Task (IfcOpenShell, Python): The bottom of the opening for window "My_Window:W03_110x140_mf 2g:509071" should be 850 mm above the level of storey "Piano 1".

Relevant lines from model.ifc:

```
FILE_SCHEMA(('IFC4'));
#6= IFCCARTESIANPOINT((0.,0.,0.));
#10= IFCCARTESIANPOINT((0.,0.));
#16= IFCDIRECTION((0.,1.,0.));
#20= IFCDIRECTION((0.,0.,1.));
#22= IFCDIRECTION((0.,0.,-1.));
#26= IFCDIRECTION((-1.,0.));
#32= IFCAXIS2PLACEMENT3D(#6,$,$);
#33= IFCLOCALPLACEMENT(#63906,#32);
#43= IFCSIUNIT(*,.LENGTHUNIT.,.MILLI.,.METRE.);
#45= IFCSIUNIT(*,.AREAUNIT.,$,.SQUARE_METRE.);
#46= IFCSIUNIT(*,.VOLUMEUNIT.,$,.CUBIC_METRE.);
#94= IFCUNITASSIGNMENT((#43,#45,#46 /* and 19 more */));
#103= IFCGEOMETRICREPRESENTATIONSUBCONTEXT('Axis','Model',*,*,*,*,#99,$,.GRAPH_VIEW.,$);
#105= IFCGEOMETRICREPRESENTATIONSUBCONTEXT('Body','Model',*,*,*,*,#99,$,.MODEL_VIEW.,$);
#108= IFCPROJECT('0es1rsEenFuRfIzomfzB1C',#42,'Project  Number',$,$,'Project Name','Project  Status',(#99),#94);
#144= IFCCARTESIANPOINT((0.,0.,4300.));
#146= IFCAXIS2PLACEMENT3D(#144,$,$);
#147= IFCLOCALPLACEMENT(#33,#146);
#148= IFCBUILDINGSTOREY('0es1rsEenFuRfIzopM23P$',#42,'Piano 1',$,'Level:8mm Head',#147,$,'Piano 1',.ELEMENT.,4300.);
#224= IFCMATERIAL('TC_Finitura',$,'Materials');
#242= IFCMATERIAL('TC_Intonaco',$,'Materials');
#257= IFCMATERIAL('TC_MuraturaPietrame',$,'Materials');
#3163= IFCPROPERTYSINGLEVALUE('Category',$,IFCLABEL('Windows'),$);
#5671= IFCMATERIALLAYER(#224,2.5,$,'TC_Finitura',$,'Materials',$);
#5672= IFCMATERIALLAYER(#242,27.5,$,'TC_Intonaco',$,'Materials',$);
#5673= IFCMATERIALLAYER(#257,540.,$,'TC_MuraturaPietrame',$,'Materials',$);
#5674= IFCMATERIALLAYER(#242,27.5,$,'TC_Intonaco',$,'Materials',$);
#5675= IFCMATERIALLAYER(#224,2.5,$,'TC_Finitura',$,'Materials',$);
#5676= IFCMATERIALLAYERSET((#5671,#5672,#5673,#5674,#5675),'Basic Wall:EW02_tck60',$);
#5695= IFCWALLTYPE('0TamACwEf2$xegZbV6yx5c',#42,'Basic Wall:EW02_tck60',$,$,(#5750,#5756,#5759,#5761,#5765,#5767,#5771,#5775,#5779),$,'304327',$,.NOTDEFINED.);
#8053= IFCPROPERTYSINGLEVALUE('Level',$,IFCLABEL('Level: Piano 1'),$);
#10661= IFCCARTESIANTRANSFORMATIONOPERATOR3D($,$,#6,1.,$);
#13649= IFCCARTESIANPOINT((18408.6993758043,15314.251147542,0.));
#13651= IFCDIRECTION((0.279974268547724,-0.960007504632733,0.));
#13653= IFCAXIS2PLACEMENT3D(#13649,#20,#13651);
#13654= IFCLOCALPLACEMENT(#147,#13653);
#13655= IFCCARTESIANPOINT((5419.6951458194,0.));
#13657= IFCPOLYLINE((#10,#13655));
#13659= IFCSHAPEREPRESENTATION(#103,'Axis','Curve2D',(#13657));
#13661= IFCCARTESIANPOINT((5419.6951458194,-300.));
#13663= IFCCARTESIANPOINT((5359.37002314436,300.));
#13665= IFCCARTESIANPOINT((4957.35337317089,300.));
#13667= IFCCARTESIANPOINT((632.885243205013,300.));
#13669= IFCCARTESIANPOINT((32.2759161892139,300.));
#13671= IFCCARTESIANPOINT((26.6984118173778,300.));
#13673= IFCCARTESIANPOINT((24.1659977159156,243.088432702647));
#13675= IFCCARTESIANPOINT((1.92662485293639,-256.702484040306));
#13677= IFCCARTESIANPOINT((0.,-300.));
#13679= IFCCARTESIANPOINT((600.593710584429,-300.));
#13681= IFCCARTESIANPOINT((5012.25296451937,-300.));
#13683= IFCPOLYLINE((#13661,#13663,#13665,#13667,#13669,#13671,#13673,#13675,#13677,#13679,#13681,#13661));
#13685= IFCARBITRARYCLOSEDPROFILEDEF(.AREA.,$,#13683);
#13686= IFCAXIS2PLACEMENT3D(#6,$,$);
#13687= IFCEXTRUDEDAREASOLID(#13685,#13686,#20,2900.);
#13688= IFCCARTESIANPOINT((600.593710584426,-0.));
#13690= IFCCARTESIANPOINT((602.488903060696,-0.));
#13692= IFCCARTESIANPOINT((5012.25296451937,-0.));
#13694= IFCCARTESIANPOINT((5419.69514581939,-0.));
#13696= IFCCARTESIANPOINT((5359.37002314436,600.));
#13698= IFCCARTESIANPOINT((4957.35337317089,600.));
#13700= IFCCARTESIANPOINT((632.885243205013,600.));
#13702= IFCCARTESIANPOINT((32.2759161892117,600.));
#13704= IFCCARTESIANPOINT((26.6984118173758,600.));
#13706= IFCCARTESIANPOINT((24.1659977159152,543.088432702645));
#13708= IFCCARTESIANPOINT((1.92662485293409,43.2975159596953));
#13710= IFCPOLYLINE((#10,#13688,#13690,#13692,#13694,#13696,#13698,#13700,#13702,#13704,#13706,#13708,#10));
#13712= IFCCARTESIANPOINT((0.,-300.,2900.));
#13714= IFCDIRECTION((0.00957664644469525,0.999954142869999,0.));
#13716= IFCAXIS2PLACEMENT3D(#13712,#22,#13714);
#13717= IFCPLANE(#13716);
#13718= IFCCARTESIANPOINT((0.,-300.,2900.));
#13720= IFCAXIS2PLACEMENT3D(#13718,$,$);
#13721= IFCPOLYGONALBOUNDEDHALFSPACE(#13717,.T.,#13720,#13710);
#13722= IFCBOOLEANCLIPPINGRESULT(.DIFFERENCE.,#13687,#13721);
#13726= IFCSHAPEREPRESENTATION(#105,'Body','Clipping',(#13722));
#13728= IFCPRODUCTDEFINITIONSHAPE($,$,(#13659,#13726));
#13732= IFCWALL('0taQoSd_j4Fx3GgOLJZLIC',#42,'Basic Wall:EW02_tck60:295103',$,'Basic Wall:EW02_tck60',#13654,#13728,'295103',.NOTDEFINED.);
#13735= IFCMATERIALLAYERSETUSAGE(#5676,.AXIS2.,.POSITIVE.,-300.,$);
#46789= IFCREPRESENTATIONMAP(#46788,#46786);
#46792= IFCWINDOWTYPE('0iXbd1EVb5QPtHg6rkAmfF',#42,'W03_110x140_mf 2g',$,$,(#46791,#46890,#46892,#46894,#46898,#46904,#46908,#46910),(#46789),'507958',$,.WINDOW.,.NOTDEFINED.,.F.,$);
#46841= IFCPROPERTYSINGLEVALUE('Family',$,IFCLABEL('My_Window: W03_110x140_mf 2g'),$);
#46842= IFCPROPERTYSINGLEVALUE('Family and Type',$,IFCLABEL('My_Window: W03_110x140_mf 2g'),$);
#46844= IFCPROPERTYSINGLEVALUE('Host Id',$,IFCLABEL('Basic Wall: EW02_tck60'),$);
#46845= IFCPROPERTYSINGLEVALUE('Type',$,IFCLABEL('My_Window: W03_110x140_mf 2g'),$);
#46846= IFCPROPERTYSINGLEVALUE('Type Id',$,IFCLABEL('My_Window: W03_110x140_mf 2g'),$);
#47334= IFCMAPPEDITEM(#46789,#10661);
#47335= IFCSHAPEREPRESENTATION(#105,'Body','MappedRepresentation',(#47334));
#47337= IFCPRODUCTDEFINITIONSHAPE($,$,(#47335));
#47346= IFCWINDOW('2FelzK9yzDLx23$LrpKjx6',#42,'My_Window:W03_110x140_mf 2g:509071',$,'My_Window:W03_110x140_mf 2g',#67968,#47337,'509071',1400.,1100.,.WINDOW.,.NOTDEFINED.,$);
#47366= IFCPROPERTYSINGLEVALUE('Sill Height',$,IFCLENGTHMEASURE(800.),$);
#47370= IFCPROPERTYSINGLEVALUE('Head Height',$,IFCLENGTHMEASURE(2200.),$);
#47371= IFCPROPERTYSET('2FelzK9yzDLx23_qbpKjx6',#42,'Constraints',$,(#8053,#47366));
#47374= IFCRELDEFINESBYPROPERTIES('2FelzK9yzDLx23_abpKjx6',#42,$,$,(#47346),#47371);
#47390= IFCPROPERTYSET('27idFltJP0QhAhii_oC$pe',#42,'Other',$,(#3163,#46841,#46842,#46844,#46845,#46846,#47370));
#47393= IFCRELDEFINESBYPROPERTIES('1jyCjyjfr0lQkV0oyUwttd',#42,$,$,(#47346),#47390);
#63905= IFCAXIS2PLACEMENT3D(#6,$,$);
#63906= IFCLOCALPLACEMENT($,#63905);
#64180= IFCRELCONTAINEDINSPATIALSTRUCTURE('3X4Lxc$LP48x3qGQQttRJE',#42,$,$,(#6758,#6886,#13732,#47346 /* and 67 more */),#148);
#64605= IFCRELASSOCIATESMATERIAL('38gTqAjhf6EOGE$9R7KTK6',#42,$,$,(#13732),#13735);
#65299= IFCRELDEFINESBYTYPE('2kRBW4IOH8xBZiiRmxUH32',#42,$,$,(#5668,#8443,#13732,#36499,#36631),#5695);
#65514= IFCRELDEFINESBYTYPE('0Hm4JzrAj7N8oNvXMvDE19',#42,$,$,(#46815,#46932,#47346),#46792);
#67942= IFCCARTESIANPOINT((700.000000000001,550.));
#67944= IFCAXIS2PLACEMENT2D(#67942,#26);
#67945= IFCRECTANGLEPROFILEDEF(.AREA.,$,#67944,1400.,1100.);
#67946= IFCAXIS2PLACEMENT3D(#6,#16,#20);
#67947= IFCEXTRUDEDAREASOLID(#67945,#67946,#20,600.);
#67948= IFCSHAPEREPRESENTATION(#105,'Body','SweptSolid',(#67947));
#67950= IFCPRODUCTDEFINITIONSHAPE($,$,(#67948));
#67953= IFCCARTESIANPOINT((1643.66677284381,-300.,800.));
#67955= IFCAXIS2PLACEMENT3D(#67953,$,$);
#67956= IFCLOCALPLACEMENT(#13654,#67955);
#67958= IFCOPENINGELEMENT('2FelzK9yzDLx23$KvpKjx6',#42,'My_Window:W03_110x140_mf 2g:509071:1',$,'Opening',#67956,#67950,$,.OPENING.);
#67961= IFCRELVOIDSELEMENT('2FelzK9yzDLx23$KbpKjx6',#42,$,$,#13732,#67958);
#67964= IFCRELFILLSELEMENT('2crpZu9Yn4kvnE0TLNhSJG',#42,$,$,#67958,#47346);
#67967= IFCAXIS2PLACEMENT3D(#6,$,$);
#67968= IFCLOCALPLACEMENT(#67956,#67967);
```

```python
import numpy as np
import ifcopenshell
import ifcopenshell.api.geometry
import ifcopenshell.api.pset
import ifcopenshell.geom
import ifcopenshell.util.element
import ifcopenshell.util.placement
import ifcopenshell.util.shape
import ifcopenshell.util.unit

model = ifcopenshell.open("model.ifc")
unit_scale = ifcopenshell.util.unit.calculate_unit_scale(model)

window = model.by_id(47346)
opening = window.FillsVoids[0].RelatingOpeningElement
storey = ifcopenshell.util.element.get_container(window, ifc_class="IfcBuildingStorey")
level = ifcopenshell.util.placement.get_local_placement(storey.ObjectPlacement)[2, 3]

# The opening's origin need not be at the sill, so measure its lowest point.
shape = ifcopenshell.geom.create_shape(ifcopenshell.geom.settings(), opening)
bottom = ifcopenshell.util.shape.get_shape_bottom_elevation(shape, shape.geometry) / unit_scale
dz = level + 850.0 - bottom

shift = np.array([0.0, 0.0, dz])
# The window is placed relative to its opening, so it follows when the opening moves.
matrix = ifcopenshell.util.placement.get_local_placement(opening.ObjectPlacement)
matrix[:3, 3] += shift
ifcopenshell.api.geometry.edit_object_placement(
    model, product=opening, matrix=matrix, is_si=False, should_transform_children=True
)

# Keep the stored heights in step.
pset = model.by_id(ifcopenshell.util.element.get_pset(window, "Constraints", should_inherit=False)["id"])
ifcopenshell.api.pset.edit_pset(model, pset=pset, properties={
    "Sill Height": model.create_entity("IfcLengthMeasure", ifcopenshell.util.element.get_pset(window, "Constraints", "Sill Height") + dz),
})
pset = model.by_id(ifcopenshell.util.element.get_pset(window, "Other", should_inherit=False)["id"])
ifcopenshell.api.pset.edit_pset(model, pset=pset, properties={
    "Head Height": model.create_entity("IfcLengthMeasure", ifcopenshell.util.element.get_pset(window, "Other", "Head Height") + dz),
})

print(f"moved by {dz * unit_scale:+.3f} m")

model.write("model_edited.ifc")
```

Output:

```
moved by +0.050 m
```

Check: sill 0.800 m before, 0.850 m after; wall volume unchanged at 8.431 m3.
